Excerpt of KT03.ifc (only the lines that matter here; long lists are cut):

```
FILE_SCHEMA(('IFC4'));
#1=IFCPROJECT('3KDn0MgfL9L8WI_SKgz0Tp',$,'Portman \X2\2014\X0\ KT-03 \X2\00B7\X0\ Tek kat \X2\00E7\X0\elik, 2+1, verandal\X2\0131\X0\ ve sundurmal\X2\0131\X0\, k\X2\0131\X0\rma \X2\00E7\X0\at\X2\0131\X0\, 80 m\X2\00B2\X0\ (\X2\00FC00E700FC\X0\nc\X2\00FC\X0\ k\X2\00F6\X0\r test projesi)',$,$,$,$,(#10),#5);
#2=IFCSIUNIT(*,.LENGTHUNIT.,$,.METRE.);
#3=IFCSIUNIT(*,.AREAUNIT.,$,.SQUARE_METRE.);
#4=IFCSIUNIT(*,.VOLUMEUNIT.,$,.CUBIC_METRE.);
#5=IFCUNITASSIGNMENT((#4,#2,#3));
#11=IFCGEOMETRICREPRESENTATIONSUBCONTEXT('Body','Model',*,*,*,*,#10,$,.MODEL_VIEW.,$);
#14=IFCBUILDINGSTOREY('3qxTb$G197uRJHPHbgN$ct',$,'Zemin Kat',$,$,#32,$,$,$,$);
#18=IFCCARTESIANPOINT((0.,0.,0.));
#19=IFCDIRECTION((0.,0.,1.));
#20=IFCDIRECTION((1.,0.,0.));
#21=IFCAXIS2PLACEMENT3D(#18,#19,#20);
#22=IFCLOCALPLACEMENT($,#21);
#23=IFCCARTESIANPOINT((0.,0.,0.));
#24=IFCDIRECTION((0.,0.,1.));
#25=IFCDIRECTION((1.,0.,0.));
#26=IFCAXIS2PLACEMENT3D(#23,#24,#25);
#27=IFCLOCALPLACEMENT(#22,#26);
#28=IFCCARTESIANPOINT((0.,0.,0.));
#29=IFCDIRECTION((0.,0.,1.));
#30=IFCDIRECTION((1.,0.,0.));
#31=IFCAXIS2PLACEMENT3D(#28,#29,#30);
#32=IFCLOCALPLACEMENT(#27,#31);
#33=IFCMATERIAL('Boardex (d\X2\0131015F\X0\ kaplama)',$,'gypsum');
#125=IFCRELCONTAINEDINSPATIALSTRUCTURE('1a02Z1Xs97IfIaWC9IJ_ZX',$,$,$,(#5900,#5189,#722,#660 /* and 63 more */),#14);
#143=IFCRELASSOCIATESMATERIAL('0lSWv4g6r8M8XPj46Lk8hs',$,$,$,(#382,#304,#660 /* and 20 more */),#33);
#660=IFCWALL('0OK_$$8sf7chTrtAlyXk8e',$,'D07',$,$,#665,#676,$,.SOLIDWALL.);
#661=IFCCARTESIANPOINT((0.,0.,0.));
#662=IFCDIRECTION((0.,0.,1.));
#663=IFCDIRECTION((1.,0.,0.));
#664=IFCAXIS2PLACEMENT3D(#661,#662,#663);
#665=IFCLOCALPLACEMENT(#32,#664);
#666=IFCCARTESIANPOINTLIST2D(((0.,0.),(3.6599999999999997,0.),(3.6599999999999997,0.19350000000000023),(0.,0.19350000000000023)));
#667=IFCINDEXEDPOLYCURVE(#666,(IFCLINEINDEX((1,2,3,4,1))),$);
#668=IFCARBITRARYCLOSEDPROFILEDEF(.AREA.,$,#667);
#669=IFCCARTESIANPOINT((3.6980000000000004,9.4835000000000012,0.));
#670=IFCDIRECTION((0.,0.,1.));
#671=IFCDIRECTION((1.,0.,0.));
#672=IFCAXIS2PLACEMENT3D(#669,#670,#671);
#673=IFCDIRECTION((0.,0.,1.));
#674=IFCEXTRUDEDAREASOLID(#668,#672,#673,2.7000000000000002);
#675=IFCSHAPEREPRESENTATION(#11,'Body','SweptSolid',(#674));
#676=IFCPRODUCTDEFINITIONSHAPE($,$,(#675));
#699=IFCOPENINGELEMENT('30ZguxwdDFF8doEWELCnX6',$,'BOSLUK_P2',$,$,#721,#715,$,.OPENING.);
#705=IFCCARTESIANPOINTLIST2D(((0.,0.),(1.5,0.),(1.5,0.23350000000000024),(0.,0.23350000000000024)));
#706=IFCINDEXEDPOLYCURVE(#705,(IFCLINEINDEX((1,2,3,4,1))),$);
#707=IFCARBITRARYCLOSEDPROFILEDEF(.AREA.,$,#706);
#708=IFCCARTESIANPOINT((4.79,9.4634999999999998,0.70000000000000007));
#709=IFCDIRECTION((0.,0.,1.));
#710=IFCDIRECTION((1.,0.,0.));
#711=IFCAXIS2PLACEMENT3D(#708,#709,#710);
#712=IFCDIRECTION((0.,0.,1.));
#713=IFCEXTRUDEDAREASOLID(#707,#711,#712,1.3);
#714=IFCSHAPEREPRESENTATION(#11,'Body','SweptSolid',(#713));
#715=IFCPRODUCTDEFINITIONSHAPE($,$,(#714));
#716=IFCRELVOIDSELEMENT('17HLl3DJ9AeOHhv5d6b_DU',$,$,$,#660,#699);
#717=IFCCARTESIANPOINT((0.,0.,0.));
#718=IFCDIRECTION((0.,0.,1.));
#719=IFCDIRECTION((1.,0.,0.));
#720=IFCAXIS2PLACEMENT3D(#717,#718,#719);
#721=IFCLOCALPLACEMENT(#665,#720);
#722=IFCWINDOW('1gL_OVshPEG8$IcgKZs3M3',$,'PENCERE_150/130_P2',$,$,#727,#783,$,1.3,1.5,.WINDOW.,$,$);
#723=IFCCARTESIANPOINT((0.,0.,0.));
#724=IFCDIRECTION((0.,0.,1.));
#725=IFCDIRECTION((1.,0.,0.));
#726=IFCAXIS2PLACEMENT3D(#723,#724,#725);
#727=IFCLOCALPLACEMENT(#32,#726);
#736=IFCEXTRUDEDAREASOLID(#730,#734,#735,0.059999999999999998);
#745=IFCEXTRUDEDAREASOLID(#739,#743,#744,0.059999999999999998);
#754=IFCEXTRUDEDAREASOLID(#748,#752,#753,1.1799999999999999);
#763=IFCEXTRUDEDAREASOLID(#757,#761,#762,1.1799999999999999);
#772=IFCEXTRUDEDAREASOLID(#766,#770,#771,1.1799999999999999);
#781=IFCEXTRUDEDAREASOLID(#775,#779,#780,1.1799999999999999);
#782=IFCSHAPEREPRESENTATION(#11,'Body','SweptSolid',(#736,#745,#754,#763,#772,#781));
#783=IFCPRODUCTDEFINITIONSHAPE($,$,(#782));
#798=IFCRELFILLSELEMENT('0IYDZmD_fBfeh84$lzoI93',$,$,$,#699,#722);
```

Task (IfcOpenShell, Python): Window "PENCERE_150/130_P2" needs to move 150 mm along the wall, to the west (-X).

```python
import ifcopenshell
import ifcopenshell.api.geometry
import ifcopenshell.util.placement
import ifcopenshell.util.unit

model = ifcopenshell.open("KT03.ifc")
unit_scale = ifcopenshell.util.unit.calculate_unit_scale(model)

window = model.by_id(722)
opening = window.FillsVoids[0].RelatingOpeningElement
wall = opening.VoidsElements[0].RelatingBuildingElement

wall_matrix = ifcopenshell.util.placement.get_local_placement(wall.ObjectPlacement)
shift = wall_matrix[:3, 0] * -0.15 / unit_scale
before = ifcopenshell.util.placement.get_local_placement(window.ObjectPlacement)[:3, 3].copy()

# The window is not placed relative to its opening, so move both.
for product in (opening, window):
    matrix = ifcopenshell.util.placement.get_local_placement(product.ObjectPlacement)
    matrix[:3, 3] += shift
    ifcopenshell.api.geometry.edit_object_placement(model, product=product, matrix=matrix, is_si=False)

after = ifcopenshell.util.placement.get_local_placement(window.ObjectPlacement)[:3, 3]
print("window moved by", (after - before).round(3) + 0.0)

model.write("KT03_rev.ifc")
```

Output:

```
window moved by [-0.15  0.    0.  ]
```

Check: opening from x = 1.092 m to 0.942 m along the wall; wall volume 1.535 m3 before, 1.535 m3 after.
